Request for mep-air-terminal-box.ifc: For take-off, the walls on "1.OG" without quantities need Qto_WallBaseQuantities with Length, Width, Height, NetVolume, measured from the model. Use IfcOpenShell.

First a look at what the model holds.

```python
import ifcopenshell
import ifcopenshell.util.element
import ifcopenshell.util.unit

model = ifcopenshell.open("mep-air-terminal-box.ifc")
print(model.schema)
for unit_type in ("LENGTHUNIT", "AREAUNIT", "VOLUMEUNIT"):
    print(unit_type, ifcopenshell.util.unit.calculate_unit_scale(model, unit_type))
storey = next(s for s in model.by_type("IfcBuildingStorey") if s.Name == "1.OG")
walls = [e for e in ifcopenshell.util.element.get_decomposition(storey) if e.is_a("IfcWall")]
for e in sorted(walls, key=lambda e: e.id()):
    print(e.id(), e.is_a(), e.Name, list(ifcopenshell.util.element.get_psets(e, qtos_only=True)), sep=" | ")
```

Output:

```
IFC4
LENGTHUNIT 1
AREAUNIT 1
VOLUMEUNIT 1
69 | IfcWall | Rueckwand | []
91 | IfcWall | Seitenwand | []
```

```python
import ifcopenshell
import ifcopenshell.api.pset
import ifcopenshell.geom
import ifcopenshell.util.element
import ifcopenshell.util.shape
import ifcopenshell.util.unit

model = ifcopenshell.open("mep-air-terminal-box.ifc")
unit_scale = ifcopenshell.util.unit.calculate_unit_scale(model)
volume_scale = ifcopenshell.util.unit.calculate_unit_scale(model, "VOLUMEUNIT")
settings = ifcopenshell.geom.settings()

storey = next(s for s in model.by_type("IfcBuildingStorey") if s.Name == "1.OG")
walls = [e for e in ifcopenshell.util.element.get_decomposition(storey) if e.is_a("IfcWall")]

for e in sorted(walls, key=lambda e: e.id()):
    if ifcopenshell.util.element.get_psets(e, qtos_only=True, should_inherit=False):
        continue
    # Geometry comes back in metres, in the element's own axes.
    shape = ifcopenshell.geom.create_shape(settings, e)
    values = {
        "Length": ifcopenshell.util.shape.get_x(shape.geometry) / unit_scale,
        "Width": ifcopenshell.util.shape.get_y(shape.geometry) / unit_scale,
        "Height": ifcopenshell.util.shape.get_z(shape.geometry) / unit_scale,
        "NetVolume": ifcopenshell.util.shape.get_volume(shape.geometry) / volume_scale,
    }
    qto = ifcopenshell.api.pset.add_qto(model, product=e, name="Qto_WallBaseQuantities")
    ifcopenshell.api.pset.edit_qto(model, qto=qto, properties=values)
    print(e.id(), {k: round(v, 3) for k, v in values.items()})

model.write("mep-air-terminal-box_rev.ifc")
```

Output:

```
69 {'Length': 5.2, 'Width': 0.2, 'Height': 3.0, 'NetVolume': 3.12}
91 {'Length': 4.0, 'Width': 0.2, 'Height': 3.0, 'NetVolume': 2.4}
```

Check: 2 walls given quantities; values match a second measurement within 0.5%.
